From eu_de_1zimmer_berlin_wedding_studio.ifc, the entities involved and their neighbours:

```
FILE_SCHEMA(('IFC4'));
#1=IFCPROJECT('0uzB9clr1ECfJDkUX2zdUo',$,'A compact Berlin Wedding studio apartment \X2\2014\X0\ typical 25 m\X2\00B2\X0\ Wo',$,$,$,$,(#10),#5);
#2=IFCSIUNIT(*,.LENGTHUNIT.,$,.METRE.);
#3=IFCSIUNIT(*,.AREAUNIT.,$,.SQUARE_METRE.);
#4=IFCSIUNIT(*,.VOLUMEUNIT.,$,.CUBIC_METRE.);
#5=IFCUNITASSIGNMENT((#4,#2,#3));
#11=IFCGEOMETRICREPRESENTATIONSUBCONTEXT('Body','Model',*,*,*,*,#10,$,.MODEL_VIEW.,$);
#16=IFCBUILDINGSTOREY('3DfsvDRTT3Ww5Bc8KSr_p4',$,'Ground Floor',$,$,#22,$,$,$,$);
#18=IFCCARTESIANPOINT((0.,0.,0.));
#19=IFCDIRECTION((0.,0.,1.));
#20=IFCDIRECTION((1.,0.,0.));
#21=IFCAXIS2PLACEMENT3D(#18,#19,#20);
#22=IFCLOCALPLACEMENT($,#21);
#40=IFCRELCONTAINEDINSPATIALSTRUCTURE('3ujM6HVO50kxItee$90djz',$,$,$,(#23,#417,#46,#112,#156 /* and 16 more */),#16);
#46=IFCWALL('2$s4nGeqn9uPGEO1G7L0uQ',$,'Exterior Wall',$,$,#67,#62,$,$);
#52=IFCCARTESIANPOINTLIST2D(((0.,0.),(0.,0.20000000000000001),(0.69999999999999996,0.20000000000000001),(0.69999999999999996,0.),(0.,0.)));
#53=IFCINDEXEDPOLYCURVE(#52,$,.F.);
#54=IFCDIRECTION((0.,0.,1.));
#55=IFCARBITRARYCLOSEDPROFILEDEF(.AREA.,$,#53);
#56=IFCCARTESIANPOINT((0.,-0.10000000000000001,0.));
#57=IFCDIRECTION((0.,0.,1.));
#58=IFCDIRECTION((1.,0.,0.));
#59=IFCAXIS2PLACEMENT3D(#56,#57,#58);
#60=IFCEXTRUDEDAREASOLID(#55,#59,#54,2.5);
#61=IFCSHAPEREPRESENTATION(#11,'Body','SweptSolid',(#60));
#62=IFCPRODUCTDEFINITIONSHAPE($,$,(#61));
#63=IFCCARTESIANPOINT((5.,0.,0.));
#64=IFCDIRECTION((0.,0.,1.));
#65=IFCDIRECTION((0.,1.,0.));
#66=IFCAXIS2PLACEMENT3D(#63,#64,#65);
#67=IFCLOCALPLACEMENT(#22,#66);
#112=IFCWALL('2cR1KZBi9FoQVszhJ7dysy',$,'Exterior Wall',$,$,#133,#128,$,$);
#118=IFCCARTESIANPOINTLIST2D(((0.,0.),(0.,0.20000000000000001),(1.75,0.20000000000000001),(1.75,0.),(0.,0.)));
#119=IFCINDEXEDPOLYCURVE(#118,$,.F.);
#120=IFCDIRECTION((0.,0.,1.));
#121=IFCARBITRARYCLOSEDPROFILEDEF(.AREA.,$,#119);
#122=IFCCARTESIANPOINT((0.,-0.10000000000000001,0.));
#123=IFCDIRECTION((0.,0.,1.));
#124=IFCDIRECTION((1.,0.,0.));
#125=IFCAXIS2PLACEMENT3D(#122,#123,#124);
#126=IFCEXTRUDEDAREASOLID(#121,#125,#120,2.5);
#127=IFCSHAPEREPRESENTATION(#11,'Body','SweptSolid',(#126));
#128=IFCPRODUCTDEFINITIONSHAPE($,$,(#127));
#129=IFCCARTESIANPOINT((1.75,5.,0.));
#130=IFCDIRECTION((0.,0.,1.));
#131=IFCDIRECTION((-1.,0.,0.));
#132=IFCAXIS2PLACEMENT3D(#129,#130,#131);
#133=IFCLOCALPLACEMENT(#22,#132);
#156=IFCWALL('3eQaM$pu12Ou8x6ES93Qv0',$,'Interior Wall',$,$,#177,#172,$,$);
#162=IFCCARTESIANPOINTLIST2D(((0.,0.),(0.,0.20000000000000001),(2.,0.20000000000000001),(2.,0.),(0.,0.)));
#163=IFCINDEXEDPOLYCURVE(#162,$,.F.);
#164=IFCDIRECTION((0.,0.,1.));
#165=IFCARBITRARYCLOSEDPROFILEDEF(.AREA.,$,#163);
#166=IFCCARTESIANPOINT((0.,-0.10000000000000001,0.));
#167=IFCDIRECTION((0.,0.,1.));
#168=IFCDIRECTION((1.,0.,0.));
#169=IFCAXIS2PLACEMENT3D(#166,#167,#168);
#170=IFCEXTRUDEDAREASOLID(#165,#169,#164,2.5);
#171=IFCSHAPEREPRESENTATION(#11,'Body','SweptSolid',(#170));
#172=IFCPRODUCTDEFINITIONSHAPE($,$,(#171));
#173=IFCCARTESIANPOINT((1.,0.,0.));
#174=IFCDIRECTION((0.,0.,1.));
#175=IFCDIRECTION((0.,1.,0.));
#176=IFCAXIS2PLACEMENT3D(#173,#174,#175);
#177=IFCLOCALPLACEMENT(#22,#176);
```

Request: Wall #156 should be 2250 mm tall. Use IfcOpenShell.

```python
import ifcopenshell
import ifcopenshell.geom
import ifcopenshell.util.representation
import ifcopenshell.util.shape

model = ifcopenshell.open("eu_de_1zimmer_berlin_wedding_studio.ifc")
settings = ifcopenshell.geom.settings()


def volume(element):
    """Net volume in cubic metres, openings subtracted."""
    shape = ifcopenshell.geom.create_shape(settings, element)
    return ifcopenshell.util.shape.get_volume(shape.geometry)


wall = model.by_guid("3eQaM$pu12Ou8x6ES93Qv0")
before = volume(wall)

body = ifcopenshell.util.representation.get_representation(wall, "Model", "Body")
solid = body.Items[0]
old_height = solid.Depth
solid.Depth = 2.25
after = volume(wall)

print(f"height {old_height:g} -> {solid.Depth:g}, volume {before:.3f} -> {after:.3f} m3")

model.write("eu_de_1zimmer_berlin_wedding_studio_v2.ifc")
```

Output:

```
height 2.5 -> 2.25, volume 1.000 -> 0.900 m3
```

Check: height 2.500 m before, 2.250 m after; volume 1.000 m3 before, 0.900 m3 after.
